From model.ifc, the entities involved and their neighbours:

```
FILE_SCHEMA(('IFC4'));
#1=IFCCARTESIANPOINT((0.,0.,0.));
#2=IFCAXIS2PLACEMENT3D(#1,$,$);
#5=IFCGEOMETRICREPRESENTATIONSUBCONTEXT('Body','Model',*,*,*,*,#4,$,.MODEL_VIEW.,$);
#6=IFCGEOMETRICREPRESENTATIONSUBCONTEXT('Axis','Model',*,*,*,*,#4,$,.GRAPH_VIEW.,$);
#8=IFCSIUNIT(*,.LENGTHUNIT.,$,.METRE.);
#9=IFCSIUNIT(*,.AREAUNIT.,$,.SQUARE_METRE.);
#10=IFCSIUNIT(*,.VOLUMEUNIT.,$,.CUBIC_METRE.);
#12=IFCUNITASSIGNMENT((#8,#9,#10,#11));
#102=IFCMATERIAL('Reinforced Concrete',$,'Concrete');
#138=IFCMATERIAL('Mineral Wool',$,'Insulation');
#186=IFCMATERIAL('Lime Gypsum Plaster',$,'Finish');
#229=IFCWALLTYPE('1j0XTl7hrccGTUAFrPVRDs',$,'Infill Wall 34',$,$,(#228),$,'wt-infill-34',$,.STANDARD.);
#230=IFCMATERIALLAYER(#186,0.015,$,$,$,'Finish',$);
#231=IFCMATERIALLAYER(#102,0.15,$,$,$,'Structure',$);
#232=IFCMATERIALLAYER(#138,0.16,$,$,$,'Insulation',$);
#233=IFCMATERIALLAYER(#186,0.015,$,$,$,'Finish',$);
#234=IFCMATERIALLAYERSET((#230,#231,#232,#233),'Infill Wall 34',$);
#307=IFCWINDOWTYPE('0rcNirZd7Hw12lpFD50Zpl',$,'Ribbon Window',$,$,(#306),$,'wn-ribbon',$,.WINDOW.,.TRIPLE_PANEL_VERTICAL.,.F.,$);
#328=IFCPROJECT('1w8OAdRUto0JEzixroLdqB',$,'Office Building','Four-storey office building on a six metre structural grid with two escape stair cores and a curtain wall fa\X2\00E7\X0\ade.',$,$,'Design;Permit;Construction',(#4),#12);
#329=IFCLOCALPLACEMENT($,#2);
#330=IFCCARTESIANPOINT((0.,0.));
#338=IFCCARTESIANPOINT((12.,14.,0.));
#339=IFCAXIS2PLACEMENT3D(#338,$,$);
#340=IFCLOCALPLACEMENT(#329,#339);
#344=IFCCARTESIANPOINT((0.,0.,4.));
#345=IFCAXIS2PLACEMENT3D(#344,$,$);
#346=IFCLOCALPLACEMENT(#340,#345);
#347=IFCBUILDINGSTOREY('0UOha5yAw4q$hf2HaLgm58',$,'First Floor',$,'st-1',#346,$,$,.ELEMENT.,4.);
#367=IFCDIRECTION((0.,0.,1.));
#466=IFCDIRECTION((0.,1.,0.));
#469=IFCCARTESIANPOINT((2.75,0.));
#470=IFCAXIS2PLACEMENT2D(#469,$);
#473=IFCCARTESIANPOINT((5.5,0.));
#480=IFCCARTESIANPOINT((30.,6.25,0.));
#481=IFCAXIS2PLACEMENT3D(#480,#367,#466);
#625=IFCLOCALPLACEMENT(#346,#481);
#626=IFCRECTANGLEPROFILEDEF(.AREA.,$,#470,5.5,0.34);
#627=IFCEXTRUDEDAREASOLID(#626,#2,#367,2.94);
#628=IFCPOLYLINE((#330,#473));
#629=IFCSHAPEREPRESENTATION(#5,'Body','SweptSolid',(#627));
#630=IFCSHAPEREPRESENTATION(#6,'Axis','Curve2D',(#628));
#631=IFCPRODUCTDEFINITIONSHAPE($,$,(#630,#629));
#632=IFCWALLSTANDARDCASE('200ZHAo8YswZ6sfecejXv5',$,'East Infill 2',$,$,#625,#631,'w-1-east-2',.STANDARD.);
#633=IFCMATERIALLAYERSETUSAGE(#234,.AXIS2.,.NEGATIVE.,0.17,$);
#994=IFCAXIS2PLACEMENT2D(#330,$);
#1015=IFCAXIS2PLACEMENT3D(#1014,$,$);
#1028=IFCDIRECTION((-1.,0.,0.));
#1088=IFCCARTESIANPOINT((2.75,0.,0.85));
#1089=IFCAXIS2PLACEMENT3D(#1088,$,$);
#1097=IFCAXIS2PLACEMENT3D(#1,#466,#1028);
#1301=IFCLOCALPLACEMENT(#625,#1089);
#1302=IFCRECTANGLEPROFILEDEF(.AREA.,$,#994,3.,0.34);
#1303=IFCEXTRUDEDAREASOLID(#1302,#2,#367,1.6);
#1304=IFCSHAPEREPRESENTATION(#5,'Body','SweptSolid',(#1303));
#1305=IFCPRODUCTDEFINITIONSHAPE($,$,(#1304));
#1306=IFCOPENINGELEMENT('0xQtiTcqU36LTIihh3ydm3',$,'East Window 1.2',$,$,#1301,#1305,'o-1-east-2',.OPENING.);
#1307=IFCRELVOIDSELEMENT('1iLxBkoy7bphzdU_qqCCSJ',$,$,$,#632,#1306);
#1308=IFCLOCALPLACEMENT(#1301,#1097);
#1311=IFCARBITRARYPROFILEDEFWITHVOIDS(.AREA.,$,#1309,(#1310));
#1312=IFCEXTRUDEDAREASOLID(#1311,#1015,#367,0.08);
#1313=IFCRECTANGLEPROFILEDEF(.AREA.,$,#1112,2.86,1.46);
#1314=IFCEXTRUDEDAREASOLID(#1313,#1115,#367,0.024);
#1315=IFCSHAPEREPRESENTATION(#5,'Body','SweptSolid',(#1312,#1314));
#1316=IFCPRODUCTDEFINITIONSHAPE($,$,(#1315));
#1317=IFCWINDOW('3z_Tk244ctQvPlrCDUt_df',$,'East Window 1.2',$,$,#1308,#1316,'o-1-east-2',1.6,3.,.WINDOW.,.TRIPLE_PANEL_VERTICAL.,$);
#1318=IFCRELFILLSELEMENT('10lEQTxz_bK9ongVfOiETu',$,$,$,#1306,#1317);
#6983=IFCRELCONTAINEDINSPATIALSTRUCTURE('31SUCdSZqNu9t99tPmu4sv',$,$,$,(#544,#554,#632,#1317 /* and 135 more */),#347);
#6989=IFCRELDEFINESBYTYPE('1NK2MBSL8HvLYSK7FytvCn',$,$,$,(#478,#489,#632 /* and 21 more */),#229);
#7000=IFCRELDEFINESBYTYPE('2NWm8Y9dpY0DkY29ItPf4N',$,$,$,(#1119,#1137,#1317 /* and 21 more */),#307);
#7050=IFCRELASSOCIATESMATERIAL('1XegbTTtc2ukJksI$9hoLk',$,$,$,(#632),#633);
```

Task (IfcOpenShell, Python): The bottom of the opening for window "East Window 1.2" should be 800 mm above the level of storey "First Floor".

```python
import numpy as np
import ifcopenshell
import ifcopenshell.api.geometry
import ifcopenshell.geom
import ifcopenshell.util.element
import ifcopenshell.util.placement
import ifcopenshell.util.shape
import ifcopenshell.util.unit

model = ifcopenshell.open("model.ifc")
unit_scale = ifcopenshell.util.unit.calculate_unit_scale(model)

window = model.by_guid("3z_Tk244ctQvPlrCDUt_df")
opening = window.FillsVoids[0].RelatingOpeningElement
storey = ifcopenshell.util.element.get_container(window, ifc_class="IfcBuildingStorey")
level = ifcopenshell.util.placement.get_local_placement(storey.ObjectPlacement)[2, 3]

# The opening's origin need not be at the sill, so measure its lowest point.
shape = ifcopenshell.geom.create_shape(ifcopenshell.geom.settings(), opening)
bottom = ifcopenshell.util.shape.get_shape_bottom_elevation(shape, shape.geometry) / unit_scale
dz = level + 0.8 - bottom

shift = np.array([0.0, 0.0, dz])
# The window is placed relative to its opening, so it follows when the opening moves.
matrix = ifcopenshell.util.placement.get_local_placement(opening.ObjectPlacement)
matrix[:3, 3] += shift
ifcopenshell.api.geometry.edit_object_placement(
    model, product=opening, matrix=matrix, is_si=False, should_transform_children=True
)

print(f"moved by {dz * unit_scale:+.3f} m")

model.write("model_rev.ifc")
```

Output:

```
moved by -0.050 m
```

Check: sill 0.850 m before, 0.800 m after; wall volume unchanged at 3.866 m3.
